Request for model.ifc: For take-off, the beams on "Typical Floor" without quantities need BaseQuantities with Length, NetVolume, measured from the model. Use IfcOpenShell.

First a look at what the model holds.

```python
import ifcopenshell
import ifcopenshell.util.element
import ifcopenshell.util.unit

model = ifcopenshell.open("model.ifc")
print(model.schema)
for unit_type in ("LENGTHUNIT", "AREAUNIT", "VOLUMEUNIT"):
    print(unit_type, ifcopenshell.util.unit.calculate_unit_scale(model, unit_type))
storey = next(s for s in model.by_type("IfcBuildingStorey") if s.Name == "Typical Floor")
beams = [e for e in ifcopenshell.util.element.get_decomposition(storey) if e.is_a("IfcBeam")]
for e in sorted(beams, key=lambda e: e.id()):
    print(e.id(), e.is_a(), e.Name, list(ifcopenshell.util.element.get_psets(e, qtos_only=True)), sep=" | ")
```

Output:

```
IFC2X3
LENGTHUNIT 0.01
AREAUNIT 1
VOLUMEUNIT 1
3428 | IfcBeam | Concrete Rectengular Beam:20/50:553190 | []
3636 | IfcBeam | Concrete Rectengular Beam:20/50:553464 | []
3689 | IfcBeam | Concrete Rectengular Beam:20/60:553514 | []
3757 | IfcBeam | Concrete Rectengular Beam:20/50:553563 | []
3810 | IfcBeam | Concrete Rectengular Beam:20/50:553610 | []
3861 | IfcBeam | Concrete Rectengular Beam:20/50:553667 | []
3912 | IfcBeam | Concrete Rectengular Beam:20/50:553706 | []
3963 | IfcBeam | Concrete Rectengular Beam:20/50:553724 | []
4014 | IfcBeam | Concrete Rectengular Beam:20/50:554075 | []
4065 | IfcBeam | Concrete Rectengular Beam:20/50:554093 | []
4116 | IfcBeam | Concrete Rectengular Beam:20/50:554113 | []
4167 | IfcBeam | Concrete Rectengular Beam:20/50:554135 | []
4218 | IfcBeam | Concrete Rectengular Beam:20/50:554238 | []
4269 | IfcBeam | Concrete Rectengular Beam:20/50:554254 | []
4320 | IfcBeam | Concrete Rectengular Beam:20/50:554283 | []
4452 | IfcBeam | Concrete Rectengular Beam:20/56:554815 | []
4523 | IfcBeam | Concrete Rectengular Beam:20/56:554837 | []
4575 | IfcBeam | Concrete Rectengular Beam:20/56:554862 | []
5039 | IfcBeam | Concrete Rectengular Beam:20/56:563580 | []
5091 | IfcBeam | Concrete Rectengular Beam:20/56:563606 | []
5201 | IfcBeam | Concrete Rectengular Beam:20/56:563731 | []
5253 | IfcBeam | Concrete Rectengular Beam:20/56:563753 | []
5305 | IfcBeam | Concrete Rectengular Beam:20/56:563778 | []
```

```python
import ifcopenshell
import ifcopenshell.api.pset
import ifcopenshell.geom
import ifcopenshell.util.element
import ifcopenshell.util.shape
import ifcopenshell.util.unit

model = ifcopenshell.open("model.ifc")
unit_scale = ifcopenshell.util.unit.calculate_unit_scale(model)
volume_scale = ifcopenshell.util.unit.calculate_unit_scale(model, "VOLUMEUNIT")
settings = ifcopenshell.geom.settings()

storey = next(s for s in model.by_type("IfcBuildingStorey") if s.Name == "Typical Floor")
beams = [e for e in ifcopenshell.util.element.get_decomposition(storey) if e.is_a("IfcBeam")]

for e in sorted(beams, key=lambda e: e.id()):
    if ifcopenshell.util.element.get_psets(e, qtos_only=True, should_inherit=False):
        continue
    # Geometry comes back in metres, in the element's own axes.
    shape = ifcopenshell.geom.create_shape(settings, e)
    values = {
        "Length": ifcopenshell.util.shape.get_max_xyz(shape.geometry) / unit_scale,
        "NetVolume": ifcopenshell.util.shape.get_volume(shape.geometry) / volume_scale,
    }
    qto = ifcopenshell.api.pset.add_qto(model, product=e, name="BaseQuantities")
    ifcopenshell.api.pset.edit_qto(model, qto=qto, properties=values)
    print(e.id(), {k: round(v, 3) for k, v in values.items()})

model.write("model_edited.ifc")
```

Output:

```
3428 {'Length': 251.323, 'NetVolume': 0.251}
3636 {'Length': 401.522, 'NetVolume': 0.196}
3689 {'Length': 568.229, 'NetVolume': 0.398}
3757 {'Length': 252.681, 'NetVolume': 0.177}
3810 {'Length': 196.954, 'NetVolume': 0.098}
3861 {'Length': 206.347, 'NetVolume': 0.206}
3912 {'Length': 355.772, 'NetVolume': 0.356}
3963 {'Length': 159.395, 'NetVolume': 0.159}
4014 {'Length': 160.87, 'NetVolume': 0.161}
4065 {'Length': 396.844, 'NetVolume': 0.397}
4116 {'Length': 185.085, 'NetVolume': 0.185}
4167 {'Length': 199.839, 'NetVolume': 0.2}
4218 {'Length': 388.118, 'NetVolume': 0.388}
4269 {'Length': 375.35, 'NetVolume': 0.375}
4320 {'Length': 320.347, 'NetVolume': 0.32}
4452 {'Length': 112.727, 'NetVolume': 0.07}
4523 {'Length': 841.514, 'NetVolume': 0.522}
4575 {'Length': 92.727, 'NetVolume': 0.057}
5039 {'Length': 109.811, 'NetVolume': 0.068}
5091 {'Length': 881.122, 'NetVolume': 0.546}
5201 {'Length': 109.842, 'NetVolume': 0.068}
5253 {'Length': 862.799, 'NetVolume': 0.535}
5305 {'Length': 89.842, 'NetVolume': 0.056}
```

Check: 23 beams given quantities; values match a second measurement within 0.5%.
